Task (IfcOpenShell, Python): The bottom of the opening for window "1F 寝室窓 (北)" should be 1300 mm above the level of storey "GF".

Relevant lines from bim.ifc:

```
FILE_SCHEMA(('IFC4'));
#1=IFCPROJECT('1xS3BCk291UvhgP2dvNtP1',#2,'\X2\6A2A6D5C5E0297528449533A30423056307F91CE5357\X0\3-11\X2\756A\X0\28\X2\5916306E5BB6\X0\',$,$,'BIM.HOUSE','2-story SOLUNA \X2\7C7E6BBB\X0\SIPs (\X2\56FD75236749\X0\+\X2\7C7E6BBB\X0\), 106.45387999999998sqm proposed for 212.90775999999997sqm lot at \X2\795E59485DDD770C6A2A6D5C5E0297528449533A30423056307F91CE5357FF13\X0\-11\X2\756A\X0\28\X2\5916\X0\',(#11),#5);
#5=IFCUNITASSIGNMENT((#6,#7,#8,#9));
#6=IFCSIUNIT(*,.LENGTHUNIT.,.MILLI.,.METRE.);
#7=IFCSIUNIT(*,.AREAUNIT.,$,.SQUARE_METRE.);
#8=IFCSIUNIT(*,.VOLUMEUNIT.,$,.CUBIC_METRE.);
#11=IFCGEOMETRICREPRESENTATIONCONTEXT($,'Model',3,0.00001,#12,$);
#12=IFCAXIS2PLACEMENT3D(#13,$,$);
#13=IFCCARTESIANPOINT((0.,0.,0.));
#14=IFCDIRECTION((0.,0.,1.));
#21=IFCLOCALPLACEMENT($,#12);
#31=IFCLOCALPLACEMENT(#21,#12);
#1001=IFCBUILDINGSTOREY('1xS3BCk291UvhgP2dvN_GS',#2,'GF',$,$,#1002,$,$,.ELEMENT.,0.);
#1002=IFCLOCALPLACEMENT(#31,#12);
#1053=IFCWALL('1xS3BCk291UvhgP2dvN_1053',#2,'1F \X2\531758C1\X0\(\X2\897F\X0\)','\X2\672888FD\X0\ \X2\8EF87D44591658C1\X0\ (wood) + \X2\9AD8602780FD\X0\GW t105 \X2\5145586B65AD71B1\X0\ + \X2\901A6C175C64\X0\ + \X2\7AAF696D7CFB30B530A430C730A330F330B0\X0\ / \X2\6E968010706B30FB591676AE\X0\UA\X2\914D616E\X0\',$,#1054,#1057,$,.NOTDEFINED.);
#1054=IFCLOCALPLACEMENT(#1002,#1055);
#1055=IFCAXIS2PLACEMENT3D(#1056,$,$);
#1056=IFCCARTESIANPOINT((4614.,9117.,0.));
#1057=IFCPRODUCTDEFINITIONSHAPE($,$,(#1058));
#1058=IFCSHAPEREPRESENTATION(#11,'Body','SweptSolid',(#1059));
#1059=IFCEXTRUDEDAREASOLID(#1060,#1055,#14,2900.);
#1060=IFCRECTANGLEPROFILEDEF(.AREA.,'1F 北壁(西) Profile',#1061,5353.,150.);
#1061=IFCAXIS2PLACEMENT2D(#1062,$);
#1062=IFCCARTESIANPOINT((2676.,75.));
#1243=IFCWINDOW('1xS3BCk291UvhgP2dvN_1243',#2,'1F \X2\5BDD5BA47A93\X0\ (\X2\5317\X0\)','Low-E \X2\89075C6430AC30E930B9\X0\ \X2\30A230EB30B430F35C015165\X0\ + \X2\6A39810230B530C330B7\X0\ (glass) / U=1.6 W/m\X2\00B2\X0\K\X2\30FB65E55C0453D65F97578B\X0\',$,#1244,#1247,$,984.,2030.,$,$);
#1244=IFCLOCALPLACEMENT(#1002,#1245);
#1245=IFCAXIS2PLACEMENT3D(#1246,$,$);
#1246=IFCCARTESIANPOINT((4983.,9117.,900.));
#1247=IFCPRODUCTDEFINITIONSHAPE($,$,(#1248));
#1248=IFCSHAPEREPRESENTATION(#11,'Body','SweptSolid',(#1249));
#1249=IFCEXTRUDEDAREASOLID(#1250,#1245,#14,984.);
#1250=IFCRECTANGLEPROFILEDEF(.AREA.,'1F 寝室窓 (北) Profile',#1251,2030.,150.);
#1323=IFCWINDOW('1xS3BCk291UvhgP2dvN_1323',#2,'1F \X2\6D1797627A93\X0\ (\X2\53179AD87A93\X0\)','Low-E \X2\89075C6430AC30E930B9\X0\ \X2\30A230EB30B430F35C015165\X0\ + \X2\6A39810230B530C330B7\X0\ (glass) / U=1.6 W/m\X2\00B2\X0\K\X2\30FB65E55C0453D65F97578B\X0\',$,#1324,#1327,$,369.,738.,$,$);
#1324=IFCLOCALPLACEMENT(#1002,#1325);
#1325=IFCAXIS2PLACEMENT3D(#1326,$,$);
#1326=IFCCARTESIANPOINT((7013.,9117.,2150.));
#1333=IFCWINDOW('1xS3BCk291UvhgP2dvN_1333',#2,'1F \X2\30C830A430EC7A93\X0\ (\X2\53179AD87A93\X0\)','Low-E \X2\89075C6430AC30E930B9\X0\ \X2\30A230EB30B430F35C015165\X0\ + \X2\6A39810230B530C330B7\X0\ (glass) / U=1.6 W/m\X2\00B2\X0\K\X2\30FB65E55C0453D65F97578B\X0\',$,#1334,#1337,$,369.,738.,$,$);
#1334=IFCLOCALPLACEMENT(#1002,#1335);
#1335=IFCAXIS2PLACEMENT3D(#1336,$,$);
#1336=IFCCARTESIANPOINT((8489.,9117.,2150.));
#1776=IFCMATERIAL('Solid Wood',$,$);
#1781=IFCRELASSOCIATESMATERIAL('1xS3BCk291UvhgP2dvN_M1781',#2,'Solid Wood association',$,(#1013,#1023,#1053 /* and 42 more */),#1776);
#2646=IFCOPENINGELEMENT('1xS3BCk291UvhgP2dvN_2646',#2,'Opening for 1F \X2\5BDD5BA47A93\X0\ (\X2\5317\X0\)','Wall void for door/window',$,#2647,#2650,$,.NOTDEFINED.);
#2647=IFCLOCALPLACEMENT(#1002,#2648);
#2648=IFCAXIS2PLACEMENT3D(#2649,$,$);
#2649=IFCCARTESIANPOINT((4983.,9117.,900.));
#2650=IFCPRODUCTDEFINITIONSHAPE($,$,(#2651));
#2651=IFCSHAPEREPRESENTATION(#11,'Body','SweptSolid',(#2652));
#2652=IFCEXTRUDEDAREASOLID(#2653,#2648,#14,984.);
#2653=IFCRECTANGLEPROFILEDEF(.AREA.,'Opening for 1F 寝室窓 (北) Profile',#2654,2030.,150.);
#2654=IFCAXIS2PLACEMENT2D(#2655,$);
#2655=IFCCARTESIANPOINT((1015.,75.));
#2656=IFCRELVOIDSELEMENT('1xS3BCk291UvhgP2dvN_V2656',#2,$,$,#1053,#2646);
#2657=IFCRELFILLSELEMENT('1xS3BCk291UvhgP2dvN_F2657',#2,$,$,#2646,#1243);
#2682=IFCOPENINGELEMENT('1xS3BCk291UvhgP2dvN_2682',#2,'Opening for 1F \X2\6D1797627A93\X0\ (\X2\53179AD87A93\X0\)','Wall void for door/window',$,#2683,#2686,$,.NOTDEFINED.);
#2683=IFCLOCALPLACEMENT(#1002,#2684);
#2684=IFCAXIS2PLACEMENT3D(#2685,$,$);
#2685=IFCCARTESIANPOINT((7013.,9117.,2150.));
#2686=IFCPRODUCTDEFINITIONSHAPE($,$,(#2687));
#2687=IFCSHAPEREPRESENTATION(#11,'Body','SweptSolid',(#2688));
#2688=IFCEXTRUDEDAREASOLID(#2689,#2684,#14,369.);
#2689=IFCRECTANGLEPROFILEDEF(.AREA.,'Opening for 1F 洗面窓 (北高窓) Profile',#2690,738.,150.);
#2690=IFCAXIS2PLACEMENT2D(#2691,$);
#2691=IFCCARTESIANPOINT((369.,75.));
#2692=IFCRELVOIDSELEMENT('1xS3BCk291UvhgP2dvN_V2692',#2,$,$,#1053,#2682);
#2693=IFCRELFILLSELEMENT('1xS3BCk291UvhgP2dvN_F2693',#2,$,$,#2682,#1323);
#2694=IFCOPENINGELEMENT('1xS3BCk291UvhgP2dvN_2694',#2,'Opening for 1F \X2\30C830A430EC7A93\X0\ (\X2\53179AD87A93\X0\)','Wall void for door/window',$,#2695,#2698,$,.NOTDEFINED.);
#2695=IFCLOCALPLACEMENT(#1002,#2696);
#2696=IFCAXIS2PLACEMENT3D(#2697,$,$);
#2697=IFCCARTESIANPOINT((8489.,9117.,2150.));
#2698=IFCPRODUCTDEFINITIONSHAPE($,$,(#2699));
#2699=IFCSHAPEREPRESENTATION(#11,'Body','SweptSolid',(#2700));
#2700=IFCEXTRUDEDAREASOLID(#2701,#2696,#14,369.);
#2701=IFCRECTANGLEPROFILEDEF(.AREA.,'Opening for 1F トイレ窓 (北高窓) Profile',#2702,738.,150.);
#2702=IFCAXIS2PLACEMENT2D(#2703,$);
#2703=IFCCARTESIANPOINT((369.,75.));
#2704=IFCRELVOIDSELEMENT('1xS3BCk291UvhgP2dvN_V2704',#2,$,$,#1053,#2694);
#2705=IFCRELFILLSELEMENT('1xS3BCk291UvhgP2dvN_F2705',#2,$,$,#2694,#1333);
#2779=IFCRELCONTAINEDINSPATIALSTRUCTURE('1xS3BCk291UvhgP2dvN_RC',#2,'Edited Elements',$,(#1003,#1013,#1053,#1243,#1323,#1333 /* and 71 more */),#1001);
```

```python
import numpy as np
import ifcopenshell
import ifcopenshell.api.geometry
import ifcopenshell.geom
import ifcopenshell.util.element
import ifcopenshell.util.placement
import ifcopenshell.util.shape
import ifcopenshell.util.unit

model = ifcopenshell.open("bim.ifc")
unit_scale = ifcopenshell.util.unit.calculate_unit_scale(model)

window = model.by_id(1243)
opening = window.FillsVoids[0].RelatingOpeningElement
storey = ifcopenshell.util.element.get_container(window, ifc_class="IfcBuildingStorey")
level = ifcopenshell.util.placement.get_local_placement(storey.ObjectPlacement)[2, 3]

# The opening's origin need not be at the sill, so measure its lowest point.
shape = ifcopenshell.geom.create_shape(ifcopenshell.geom.settings(), opening)
bottom = ifcopenshell.util.shape.get_shape_bottom_elevation(shape, shape.geometry) / unit_scale
dz = level + 1300.0 - bottom

shift = np.array([0.0, 0.0, dz])
# The window is not placed relative to its opening, so move both.
for product in (opening, window):
    matrix = ifcopenshell.util.placement.get_local_placement(product.ObjectPlacement)
    matrix[:3, 3] += shift
    ifcopenshell.api.geometry.edit_object_placement(model, product=product, matrix=matrix, is_si=False)

print(f"moved by {dz * unit_scale:+.3f} m")

model.write("bim_rev.ifc")
```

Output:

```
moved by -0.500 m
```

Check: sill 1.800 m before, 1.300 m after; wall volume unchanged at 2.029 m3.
